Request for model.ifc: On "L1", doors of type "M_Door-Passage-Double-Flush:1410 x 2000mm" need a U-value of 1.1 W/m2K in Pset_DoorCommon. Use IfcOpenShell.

First a look at what the model holds.

```python
import ifcopenshell
import ifcopenshell.util.element

model = ifcopenshell.open("model.ifc")
print(model.schema)
storey = next(s for s in model.by_type("IfcBuildingStorey") if s.Name == "L1")
doors = [e for e in ifcopenshell.util.element.get_decomposition(storey) if e.is_a("IfcDoor")]
seen = {}
for e in doors:
    element_type = ifcopenshell.util.element.get_type(e)
    key = (element_type.Name if element_type != e and element_type else None, ifcopenshell.util.element.get_pset(e, "Pset_DoorCommon", "ThermalTransmittance"))
    seen[key] = seen.get(key, 0) + 1
for (name, value), count in sorted(seen.items(), key=str):
    print(count, "x", name, "|", value)
```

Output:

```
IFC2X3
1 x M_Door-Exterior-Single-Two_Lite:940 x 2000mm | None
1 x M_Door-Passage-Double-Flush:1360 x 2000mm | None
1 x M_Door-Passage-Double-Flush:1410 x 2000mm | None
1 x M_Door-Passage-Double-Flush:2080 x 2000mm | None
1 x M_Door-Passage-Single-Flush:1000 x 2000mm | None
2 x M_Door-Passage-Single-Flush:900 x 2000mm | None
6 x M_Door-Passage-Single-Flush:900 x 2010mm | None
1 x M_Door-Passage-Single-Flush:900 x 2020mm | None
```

```python
import ifcopenshell
import ifcopenshell.api.pset
import ifcopenshell.util.element

model = ifcopenshell.open("model.ifc")

storey = next(s for s in model.by_type("IfcBuildingStorey") if s.Name == "L1")
doors = [e for e in ifcopenshell.util.element.get_decomposition(storey) if e.is_a("IfcDoor")]

count = 0
for e in doors:
    element_type = ifcopenshell.util.element.get_type(e)
    if element_type in (None, e) or element_type.Name != "M_Door-Passage-Double-Flush:1410 x 2000mm":
        continue
    # add_pset returns the element's existing set when there is one.
    pset = ifcopenshell.api.pset.add_pset(model, product=e, name="Pset_DoorCommon")
    ifcopenshell.api.pset.edit_pset(model, pset=pset, properties={"ThermalTransmittance": 1.1})
    count += 1

print(count, "doors updated")

model.write("model_v2.ifc")
```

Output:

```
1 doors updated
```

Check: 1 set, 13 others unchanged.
